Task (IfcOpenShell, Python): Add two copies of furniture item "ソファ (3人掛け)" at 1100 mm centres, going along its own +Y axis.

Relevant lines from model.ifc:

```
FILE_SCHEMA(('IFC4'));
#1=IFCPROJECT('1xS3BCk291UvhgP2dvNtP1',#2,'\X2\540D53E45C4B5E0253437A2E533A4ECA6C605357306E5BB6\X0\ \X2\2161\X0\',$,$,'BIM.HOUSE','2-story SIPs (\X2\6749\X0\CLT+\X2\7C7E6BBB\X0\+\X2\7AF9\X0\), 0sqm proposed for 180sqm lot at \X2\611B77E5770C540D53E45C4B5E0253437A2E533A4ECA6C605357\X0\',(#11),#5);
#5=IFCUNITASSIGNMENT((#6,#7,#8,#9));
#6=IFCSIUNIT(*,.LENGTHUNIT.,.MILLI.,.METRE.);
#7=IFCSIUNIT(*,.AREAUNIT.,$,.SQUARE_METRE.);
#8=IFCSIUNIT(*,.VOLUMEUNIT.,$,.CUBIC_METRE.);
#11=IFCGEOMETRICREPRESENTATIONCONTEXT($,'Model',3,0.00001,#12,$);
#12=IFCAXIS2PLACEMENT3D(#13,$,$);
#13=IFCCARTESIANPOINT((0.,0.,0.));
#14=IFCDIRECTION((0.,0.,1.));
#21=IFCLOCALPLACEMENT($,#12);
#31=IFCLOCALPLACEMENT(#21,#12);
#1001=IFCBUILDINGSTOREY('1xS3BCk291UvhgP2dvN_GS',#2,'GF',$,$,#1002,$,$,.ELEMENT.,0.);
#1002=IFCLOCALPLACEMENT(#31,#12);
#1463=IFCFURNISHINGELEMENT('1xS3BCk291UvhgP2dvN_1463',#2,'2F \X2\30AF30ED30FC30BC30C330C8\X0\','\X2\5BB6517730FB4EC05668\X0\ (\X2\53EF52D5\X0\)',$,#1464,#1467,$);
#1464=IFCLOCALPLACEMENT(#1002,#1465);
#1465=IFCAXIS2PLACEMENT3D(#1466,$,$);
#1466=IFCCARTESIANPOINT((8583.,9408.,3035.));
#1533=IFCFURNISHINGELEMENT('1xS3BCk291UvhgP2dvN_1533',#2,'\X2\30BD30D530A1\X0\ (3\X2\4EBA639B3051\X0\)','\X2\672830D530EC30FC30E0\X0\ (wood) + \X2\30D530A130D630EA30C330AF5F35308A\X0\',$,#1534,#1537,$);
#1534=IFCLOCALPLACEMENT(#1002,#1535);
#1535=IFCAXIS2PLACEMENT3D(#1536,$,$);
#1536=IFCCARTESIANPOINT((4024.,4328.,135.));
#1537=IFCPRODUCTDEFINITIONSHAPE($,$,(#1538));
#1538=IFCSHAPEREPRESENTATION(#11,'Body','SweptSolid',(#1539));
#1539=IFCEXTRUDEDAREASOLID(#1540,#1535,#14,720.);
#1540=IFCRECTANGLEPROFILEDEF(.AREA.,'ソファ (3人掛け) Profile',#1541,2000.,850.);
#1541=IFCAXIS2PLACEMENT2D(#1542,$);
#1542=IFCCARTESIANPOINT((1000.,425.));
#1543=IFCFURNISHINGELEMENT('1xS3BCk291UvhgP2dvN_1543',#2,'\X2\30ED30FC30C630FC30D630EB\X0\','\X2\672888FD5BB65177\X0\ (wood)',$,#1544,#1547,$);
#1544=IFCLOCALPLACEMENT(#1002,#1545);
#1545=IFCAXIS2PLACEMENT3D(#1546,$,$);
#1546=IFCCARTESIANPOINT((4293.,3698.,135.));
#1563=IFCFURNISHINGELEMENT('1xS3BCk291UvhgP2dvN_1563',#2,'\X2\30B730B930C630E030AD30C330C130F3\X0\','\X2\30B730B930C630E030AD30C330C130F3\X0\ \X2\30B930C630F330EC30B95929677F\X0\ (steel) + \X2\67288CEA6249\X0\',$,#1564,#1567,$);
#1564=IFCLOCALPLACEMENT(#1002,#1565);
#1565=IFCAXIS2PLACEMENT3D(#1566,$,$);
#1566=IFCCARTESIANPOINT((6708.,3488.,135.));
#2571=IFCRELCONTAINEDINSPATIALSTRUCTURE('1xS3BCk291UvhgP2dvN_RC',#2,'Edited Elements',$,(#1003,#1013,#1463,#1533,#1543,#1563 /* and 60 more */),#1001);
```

```python
import ifcopenshell
import ifcopenshell.api.geometry
import ifcopenshell.api.root
import ifcopenshell.util.element
import ifcopenshell.util.placement
import ifcopenshell.util.unit

model = ifcopenshell.open("model.ifc")
unit_scale = ifcopenshell.util.unit.calculate_unit_scale(model)


def reuse_history(source, copy):
    """copy_class also copies each property set's owner history, people and application; keep the originals."""
    for rel in copy.IsDefinedBy:
        if rel.is_a("IfcRelDefinesByProperties") and (history := rel.RelatingPropertyDefinition.OwnerHistory):
            rel.RelatingPropertyDefinition.OwnerHistory = source.OwnerHistory
            ifcopenshell.util.element.remove_deep2(model, history)


source = model.by_guid("1xS3BCk291UvhgP2dvN_1533")
base = ifcopenshell.util.placement.get_local_placement(source.ObjectPlacement)
step = base[:3, 1] * 1.1 / unit_scale

for i in range(1, 3):
    copy = ifcopenshell.api.root.copy_class(model, product=source)
    copy.Representation = ifcopenshell.util.element.copy_deep(
        model, source.Representation, exclude=["IfcGeometricRepresentationContext", "IfcRepresentationMap"]
    )
    reuse_history(source, copy)
    matrix = base.copy()
    matrix[:3, 3] += i * step
    print("added at", matrix[:3, 3].round(3) + 0.0)
    ifcopenshell.api.geometry.edit_object_placement(model, product=copy, matrix=matrix, is_si=False)

model.write("model_edited.ifc")
```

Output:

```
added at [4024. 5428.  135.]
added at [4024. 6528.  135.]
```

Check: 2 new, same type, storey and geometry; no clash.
